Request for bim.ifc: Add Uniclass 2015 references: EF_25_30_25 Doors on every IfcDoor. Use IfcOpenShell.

First a look at what the model holds.

```python
import ifcopenshell

model = ifcopenshell.open("bim.ifc")
print(model.schema)
print("classifications:", [c.Name for c in model.by_type("IfcClassification")])
for ifc_class in ("IfcDoor", "IfcRoof", "IfcStair", "IfcWall", "IfcWindow"):
    print(ifc_class, len(model.by_type(ifc_class)))
```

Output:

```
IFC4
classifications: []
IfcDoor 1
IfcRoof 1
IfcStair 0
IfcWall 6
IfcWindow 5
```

```python
import ifcopenshell
import ifcopenshell.api.classification

model = ifcopenshell.open("bim.ifc")

system = ifcopenshell.api.classification.add_classification(model, classification="Uniclass 2015")

codes = {
    "IfcDoor": ("EF_25_30_25", "Doors"),
}
for ifc_class, (code, name) in codes.items():
    products = model.by_type(ifc_class)
    ifcopenshell.api.classification.add_reference(
        model, products=products, classification=system, identification=code, name=name
    )
    print(code, len(products))

model.write("bim_v2.ifc")
```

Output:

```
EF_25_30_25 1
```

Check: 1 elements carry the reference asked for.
